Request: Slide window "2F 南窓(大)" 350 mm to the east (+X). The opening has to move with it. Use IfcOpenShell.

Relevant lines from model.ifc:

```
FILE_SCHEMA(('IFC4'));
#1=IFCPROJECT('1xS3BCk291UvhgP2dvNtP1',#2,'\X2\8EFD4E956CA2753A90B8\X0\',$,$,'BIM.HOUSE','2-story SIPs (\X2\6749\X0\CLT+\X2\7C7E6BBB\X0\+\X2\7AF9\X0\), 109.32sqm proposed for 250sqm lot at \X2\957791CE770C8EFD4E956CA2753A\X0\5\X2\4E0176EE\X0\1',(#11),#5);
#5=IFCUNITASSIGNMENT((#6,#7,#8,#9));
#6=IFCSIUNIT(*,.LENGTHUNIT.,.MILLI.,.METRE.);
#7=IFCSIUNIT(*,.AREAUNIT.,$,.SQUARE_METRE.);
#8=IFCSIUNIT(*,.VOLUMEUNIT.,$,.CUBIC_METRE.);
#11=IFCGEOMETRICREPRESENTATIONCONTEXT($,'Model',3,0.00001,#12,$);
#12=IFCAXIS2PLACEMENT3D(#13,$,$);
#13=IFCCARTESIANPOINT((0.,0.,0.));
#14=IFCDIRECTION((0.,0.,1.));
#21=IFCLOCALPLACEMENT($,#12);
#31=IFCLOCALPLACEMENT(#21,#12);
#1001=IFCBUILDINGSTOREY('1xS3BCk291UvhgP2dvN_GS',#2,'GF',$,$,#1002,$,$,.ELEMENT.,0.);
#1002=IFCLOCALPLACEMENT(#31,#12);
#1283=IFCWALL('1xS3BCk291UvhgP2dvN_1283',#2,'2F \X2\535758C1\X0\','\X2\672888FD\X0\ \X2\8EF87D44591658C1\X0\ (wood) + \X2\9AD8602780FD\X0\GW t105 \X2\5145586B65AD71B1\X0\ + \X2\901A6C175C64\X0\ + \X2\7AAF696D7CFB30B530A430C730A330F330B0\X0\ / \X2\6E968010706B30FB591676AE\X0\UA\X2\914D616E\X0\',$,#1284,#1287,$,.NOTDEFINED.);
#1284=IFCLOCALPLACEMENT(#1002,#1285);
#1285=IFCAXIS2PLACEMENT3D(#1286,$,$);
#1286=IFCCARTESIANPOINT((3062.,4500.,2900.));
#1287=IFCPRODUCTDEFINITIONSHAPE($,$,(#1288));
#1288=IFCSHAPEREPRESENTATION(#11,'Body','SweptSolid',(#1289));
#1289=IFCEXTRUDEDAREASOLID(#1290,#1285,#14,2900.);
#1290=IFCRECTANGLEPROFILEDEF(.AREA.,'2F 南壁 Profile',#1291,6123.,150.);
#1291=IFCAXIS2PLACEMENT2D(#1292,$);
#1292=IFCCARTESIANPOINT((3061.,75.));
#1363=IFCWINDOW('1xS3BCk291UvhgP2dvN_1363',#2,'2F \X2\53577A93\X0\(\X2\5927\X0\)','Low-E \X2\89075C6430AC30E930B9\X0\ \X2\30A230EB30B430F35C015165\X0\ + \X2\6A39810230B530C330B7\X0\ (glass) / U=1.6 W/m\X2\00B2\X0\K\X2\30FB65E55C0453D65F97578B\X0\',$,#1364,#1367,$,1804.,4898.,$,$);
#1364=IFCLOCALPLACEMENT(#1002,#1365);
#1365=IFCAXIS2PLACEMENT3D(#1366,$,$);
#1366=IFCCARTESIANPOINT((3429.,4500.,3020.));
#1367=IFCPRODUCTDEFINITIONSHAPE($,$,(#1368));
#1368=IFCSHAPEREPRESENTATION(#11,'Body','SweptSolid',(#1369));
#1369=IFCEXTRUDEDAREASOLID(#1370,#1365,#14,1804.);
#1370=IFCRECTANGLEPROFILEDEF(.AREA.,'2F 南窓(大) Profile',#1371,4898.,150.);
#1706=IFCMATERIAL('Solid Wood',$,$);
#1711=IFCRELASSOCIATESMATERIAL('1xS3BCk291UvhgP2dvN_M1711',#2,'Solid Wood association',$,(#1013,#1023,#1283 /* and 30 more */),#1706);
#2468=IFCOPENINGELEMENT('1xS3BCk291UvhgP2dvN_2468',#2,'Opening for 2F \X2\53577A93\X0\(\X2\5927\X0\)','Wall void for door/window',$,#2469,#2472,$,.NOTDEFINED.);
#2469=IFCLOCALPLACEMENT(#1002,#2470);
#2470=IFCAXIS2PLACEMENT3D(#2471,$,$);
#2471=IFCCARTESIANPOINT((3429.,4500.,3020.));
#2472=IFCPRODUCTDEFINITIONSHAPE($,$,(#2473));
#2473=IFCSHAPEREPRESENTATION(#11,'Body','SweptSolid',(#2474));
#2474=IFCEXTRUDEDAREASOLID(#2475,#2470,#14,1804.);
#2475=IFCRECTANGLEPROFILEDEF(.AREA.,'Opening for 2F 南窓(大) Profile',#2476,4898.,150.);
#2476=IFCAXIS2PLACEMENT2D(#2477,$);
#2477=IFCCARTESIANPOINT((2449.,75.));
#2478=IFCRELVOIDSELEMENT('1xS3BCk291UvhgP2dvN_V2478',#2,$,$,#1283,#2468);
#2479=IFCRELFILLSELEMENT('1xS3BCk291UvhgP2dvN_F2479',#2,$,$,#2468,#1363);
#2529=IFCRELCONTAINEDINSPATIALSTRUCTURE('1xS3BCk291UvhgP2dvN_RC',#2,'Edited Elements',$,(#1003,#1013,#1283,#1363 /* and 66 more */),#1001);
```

```python
import ifcopenshell
import ifcopenshell.api.geometry
import ifcopenshell.util.placement
import ifcopenshell.util.unit

model = ifcopenshell.open("model.ifc")
unit_scale = ifcopenshell.util.unit.calculate_unit_scale(model)

window = model.by_id(1363)
opening = window.FillsVoids[0].RelatingOpeningElement
wall = opening.VoidsElements[0].RelatingBuildingElement

wall_matrix = ifcopenshell.util.placement.get_local_placement(wall.ObjectPlacement)
shift = wall_matrix[:3, 0] * 0.35 / unit_scale
before = ifcopenshell.util.placement.get_local_placement(window.ObjectPlacement)[:3, 3].copy()

# The window is not placed relative to its opening, so move both.
for product in (opening, window):
    matrix = ifcopenshell.util.placement.get_local_placement(product.ObjectPlacement)
    matrix[:3, 3] += shift
    ifcopenshell.api.geometry.edit_object_placement(model, product=product, matrix=matrix, is_si=False)

after = ifcopenshell.util.placement.get_local_placement(window.ObjectPlacement)[:3, 3]
print("window moved by", (after - before).round(3) + 0.0)

model.write("model-out.ifc")
```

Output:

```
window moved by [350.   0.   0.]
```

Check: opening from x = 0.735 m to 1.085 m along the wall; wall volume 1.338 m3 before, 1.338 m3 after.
